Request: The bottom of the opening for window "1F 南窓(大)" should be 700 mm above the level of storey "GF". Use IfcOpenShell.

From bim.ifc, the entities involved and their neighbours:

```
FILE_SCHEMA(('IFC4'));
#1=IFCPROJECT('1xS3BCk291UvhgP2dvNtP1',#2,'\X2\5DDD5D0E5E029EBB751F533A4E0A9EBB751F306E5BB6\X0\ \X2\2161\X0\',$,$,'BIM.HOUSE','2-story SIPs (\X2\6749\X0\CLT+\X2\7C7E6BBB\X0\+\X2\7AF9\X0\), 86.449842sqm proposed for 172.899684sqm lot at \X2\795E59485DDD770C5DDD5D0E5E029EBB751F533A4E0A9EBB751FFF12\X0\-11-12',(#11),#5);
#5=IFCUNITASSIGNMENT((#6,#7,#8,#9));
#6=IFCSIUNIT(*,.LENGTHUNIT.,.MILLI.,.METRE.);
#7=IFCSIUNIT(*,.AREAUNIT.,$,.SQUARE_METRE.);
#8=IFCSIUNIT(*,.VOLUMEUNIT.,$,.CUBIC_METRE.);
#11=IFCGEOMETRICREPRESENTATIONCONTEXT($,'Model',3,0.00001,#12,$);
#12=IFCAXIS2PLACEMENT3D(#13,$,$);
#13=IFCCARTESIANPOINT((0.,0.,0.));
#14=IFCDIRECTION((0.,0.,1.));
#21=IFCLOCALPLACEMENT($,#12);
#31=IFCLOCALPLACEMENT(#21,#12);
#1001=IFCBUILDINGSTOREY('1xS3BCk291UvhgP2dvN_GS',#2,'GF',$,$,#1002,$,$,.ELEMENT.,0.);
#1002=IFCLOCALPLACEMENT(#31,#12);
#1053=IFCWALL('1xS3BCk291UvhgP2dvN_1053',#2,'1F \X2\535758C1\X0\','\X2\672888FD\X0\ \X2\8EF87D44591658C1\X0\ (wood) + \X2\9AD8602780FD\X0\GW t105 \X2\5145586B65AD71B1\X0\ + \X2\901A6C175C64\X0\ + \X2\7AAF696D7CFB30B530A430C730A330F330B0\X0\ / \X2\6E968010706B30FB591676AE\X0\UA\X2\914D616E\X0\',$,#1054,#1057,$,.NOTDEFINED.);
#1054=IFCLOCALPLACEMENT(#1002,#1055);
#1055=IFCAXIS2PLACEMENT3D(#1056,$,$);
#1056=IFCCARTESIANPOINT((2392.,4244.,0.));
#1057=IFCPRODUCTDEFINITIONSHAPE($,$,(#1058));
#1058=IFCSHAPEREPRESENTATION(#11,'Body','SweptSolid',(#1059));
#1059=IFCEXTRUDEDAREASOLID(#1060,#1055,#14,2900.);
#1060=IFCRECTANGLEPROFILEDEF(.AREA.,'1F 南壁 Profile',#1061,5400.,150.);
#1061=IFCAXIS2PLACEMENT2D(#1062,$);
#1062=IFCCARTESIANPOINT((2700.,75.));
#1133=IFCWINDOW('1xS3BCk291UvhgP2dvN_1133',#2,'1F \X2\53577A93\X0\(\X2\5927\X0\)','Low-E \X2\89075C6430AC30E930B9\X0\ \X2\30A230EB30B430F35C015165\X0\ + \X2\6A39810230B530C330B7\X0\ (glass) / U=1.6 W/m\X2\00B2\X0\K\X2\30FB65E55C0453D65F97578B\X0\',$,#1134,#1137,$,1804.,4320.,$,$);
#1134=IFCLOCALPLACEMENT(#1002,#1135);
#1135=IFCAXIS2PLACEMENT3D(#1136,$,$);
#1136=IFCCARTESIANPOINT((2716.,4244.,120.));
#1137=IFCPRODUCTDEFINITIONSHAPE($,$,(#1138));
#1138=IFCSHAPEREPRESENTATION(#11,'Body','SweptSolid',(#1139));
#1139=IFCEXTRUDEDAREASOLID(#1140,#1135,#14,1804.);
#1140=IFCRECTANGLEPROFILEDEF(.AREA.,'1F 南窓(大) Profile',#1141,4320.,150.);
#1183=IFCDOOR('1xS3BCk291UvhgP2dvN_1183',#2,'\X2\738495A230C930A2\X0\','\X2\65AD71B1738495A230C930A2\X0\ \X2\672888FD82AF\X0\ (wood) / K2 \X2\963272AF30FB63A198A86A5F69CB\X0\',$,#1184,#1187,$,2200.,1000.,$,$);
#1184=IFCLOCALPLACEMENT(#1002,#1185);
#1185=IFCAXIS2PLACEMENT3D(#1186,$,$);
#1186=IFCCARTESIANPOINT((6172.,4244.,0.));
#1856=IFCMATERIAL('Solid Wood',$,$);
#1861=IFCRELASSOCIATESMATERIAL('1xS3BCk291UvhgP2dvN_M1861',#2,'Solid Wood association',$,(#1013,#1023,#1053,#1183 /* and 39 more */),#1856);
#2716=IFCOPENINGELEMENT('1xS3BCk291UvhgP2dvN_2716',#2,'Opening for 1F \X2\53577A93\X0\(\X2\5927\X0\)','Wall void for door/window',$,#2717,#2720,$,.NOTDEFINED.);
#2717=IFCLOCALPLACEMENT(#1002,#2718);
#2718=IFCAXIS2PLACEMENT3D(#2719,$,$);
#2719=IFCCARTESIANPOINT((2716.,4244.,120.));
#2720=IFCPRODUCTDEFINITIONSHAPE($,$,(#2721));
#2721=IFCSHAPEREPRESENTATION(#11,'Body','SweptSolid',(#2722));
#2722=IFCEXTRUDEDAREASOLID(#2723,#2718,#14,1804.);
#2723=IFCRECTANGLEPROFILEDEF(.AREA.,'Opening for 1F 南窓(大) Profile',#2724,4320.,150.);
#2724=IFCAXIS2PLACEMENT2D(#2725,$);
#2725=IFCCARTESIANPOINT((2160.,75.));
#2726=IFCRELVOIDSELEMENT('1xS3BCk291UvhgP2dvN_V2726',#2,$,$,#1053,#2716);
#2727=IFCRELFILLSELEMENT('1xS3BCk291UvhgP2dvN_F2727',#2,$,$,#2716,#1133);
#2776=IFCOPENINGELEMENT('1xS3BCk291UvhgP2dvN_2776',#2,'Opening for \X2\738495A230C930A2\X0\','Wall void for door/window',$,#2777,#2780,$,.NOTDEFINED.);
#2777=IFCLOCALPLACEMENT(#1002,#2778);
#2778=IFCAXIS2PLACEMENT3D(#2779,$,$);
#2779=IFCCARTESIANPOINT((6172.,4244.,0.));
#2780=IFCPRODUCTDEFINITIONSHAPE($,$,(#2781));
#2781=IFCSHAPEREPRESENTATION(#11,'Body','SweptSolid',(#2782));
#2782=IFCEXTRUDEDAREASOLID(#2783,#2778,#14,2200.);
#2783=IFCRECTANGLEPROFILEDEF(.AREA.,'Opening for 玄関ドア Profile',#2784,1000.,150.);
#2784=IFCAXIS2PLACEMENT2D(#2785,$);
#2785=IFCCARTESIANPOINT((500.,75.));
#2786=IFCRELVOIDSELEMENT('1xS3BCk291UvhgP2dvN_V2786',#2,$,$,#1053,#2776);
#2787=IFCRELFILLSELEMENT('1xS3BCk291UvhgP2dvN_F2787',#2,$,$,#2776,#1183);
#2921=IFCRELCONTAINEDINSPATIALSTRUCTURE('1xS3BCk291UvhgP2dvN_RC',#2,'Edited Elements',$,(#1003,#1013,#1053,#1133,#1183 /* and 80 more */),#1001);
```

```python
import numpy as np
import ifcopenshell
import ifcopenshell.api.geometry
import ifcopenshell.geom
import ifcopenshell.util.element
import ifcopenshell.util.placement
import ifcopenshell.util.shape
import ifcopenshell.util.unit

model = ifcopenshell.open("bim.ifc")
unit_scale = ifcopenshell.util.unit.calculate_unit_scale(model)

window = model.by_id(1133)
opening = window.FillsVoids[0].RelatingOpeningElement
storey = ifcopenshell.util.element.get_container(window, ifc_class="IfcBuildingStorey")
level = ifcopenshell.util.placement.get_local_placement(storey.ObjectPlacement)[2, 3]

# The opening's origin need not be at the sill, so measure its lowest point.
shape = ifcopenshell.geom.create_shape(ifcopenshell.geom.settings(), opening)
bottom = ifcopenshell.util.shape.get_shape_bottom_elevation(shape, shape.geometry) / unit_scale
dz = level + 0.7 / unit_scale - bottom

shift = np.array([0.0, 0.0, dz])
# The window is not placed relative to its opening, so move both.
for product in (opening, window):
    matrix = ifcopenshell.util.placement.get_local_placement(product.ObjectPlacement)
    matrix[:3, 3] += shift
    ifcopenshell.api.geometry.edit_object_placement(model, product=product, matrix=matrix, is_si=False)

print(f"moved by {dz * unit_scale:+.3f} m")

model.write("bim_v2.ifc")
```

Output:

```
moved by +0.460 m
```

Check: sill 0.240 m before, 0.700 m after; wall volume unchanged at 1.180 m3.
